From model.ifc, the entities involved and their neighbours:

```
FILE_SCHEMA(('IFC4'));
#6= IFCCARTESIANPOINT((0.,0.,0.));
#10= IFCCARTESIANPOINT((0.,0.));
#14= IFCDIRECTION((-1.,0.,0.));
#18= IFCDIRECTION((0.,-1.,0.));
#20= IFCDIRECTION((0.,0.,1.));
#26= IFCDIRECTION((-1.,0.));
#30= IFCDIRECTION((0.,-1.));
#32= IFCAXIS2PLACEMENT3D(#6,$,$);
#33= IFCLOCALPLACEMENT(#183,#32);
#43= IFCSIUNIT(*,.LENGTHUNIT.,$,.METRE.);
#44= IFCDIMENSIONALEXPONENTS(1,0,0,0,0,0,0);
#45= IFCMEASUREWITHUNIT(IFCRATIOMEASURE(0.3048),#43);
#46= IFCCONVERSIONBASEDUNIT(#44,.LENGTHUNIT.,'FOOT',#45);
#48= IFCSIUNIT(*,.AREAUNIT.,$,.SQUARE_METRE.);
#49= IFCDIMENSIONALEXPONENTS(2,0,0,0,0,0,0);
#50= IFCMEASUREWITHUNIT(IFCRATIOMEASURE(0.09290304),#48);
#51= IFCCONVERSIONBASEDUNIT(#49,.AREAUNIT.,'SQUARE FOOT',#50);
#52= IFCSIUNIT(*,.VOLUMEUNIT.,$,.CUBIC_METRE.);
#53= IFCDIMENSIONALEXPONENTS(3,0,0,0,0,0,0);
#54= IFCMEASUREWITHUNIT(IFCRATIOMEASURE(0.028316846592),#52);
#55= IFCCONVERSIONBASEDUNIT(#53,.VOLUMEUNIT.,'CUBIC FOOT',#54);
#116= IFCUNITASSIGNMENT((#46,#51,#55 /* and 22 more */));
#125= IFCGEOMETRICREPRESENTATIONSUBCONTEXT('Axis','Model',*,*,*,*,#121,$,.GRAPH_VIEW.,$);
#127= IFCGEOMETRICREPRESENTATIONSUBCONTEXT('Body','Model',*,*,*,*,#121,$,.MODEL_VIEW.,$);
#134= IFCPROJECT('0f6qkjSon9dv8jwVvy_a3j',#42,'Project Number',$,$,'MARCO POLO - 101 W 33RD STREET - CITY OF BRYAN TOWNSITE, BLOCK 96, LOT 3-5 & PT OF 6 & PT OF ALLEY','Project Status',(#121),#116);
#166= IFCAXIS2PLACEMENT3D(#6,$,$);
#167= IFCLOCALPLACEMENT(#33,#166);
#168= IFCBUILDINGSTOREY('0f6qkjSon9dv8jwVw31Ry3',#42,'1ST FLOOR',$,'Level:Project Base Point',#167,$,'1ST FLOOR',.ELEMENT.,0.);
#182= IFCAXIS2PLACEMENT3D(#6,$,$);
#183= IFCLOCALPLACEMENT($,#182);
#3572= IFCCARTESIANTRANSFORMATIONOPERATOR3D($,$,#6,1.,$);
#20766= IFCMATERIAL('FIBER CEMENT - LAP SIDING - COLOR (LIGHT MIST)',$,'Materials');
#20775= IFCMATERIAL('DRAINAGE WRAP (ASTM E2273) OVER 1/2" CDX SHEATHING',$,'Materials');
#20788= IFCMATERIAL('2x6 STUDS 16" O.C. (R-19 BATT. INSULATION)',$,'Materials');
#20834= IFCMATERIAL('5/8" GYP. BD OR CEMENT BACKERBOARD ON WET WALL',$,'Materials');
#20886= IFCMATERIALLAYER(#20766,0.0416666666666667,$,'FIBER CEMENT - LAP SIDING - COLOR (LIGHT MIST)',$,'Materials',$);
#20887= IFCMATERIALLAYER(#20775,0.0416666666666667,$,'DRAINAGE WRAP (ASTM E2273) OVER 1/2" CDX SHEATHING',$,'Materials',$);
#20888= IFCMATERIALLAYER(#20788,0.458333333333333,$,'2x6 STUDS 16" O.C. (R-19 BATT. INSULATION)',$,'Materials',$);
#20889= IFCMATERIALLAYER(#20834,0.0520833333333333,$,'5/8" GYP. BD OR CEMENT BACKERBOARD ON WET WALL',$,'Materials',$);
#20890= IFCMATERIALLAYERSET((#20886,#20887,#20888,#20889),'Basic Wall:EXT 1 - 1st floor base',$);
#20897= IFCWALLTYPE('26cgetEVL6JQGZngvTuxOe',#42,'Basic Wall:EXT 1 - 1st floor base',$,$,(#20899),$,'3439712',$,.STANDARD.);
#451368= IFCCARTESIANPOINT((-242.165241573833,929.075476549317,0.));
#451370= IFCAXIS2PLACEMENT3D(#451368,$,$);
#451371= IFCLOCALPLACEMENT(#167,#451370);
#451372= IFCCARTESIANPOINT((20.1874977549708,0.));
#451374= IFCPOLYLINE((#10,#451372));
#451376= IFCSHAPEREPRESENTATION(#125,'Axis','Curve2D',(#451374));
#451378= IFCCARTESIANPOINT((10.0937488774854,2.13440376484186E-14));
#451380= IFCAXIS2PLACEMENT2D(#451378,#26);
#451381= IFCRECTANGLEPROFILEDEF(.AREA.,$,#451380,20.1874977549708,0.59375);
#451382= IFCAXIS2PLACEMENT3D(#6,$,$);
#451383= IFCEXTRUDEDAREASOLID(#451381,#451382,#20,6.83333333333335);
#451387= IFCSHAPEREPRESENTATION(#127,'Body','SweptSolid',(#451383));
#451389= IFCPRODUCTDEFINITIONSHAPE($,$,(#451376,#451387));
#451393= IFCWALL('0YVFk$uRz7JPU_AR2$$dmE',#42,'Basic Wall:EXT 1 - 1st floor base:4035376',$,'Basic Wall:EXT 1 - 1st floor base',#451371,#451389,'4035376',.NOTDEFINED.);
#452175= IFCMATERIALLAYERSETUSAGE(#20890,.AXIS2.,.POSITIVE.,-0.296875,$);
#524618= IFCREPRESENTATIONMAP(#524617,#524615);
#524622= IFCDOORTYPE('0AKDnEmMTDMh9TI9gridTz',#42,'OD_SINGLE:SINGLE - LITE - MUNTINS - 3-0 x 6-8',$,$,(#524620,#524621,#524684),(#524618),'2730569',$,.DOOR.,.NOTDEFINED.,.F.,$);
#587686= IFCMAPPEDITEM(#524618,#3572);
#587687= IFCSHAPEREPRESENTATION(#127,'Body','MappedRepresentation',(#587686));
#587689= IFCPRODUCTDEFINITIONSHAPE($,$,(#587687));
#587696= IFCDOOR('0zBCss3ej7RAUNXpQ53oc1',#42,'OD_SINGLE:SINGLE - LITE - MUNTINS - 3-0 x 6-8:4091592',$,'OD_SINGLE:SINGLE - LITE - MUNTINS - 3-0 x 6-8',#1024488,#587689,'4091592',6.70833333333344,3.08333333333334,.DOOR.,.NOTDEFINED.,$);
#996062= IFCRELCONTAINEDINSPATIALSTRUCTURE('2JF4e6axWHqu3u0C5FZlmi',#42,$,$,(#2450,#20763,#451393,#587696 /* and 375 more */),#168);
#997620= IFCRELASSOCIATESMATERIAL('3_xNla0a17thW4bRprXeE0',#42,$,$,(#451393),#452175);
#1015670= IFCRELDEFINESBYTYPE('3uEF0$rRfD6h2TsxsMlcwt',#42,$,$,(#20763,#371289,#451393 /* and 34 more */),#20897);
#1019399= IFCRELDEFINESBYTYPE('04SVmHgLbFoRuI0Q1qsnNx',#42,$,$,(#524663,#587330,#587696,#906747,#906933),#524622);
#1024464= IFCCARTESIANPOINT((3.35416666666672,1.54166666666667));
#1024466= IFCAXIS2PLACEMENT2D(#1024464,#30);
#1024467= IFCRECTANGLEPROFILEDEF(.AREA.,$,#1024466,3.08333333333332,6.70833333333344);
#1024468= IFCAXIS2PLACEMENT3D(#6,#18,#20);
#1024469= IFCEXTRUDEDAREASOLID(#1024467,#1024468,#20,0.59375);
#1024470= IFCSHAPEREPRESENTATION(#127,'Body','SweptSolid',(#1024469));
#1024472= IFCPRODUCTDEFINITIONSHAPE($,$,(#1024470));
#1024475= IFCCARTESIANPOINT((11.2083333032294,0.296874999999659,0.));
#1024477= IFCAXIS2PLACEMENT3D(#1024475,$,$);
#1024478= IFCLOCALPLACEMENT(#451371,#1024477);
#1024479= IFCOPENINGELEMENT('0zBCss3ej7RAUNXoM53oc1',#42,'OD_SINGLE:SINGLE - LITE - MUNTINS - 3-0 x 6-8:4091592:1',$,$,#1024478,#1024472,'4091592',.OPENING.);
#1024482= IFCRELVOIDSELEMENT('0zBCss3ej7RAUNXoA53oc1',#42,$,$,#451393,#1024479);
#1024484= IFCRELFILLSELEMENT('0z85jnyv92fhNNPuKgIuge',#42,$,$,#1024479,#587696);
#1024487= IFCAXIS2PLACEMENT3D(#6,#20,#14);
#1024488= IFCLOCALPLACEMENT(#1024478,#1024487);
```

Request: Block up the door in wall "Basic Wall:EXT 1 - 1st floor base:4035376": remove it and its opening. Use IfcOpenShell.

```python
import ifcopenshell
import ifcopenshell.api.feature
import ifcopenshell.api.root
import ifcopenshell.geom
import ifcopenshell.util.shape

model = ifcopenshell.open("model.ifc")
settings = ifcopenshell.geom.settings()


def volume(element):
    """Net volume in cubic metres, openings subtracted."""
    shape = ifcopenshell.geom.create_shape(settings, element)
    return ifcopenshell.util.shape.get_volume(shape.geometry)


door = model.by_id(587696)
opening = door.FillsVoids[0].RelatingOpeningElement
wall = opening.VoidsElements[0].RelatingBuildingElement
before = volume(wall)

ifcopenshell.api.root.remove_product(model, product=door)
ifcopenshell.api.feature.remove_feature(model, feature=opening)

after = volume(wall)

print(f"wall volume {before:.3f} -> {after:.3f} m3")

model.write("model_v2.ifc")
```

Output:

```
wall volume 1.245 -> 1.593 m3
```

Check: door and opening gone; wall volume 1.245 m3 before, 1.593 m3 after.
